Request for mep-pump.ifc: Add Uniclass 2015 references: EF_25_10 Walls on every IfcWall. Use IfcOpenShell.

First a look at what the model holds.

```python
import ifcopenshell

model = ifcopenshell.open("mep-pump.ifc")
print(model.schema)
print("classifications:", [c.Name for c in model.by_type("IfcClassification")])
for ifc_class in ("IfcDoor", "IfcRoof", "IfcStair", "IfcWall", "IfcWindow"):
    print(ifc_class, len(model.by_type(ifc_class)))
```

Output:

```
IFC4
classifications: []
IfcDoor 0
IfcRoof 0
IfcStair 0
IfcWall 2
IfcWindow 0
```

```python
import ifcopenshell
import ifcopenshell.api.classification

model = ifcopenshell.open("mep-pump.ifc")

system = ifcopenshell.api.classification.add_classification(model, classification="Uniclass 2015")

codes = {
    "IfcWall": ("EF_25_10", "Walls"),
}
for ifc_class, (code, name) in codes.items():
    products = model.by_type(ifc_class)
    ifcopenshell.api.classification.add_reference(
        model, products=products, classification=system, identification=code, name=name
    )
    print(code, len(products))

model.write("mep-pump-out.ifc")
```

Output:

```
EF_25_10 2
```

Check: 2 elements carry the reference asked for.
